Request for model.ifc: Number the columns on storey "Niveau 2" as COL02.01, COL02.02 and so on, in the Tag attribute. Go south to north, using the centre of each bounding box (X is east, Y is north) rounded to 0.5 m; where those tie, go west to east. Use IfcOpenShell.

First a look at what the model holds.

```python
import ifcopenshell
import ifcopenshell.util.element
import ifcopenshell.util.placement

model = ifcopenshell.open("model.ifc")
print(model.schema)
storey = next(s for s in model.by_type("IfcBuildingStorey") if s.Name == "Niveau 2")
columns = [e for e in ifcopenshell.util.element.get_decomposition(storey) if e.is_a("IfcColumn")]
for e in sorted(columns, key=lambda e: e.id()):
    origin = ifcopenshell.util.placement.get_local_placement(e.ObjectPlacement)[:3, 3]
    print(e.id(), e.Tag, e.Name, origin.round(2) + 0.0, sep=" | ")
```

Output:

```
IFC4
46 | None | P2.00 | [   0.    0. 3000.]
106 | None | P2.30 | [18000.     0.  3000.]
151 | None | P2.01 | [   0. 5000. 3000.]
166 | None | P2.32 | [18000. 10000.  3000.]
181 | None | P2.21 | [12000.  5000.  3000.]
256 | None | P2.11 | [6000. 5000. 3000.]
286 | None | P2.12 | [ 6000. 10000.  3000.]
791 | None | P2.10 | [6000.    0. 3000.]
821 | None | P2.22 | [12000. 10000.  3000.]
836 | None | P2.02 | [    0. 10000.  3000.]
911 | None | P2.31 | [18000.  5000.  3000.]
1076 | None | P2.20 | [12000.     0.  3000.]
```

```python
import ifcopenshell
import ifcopenshell.geom
import ifcopenshell.util.element
import ifcopenshell.util.shape

model = ifcopenshell.open("model.ifc")
settings = ifcopenshell.geom.settings()
settings.set("use-world-coords", True)


def centre(element):
    shape = ifcopenshell.geom.create_shape(settings, element)
    return ifcopenshell.util.shape.get_bbox_centroid(shape.geometry)


storey = next(s for s in model.by_type("IfcBuildingStorey") if s.Name == "Niveau 2")
columns = [e for e in ifcopenshell.util.element.get_decomposition(storey) if e.is_a("IfcColumn")]

# Insertion points can sit at a corner or the storey origin, so sort by the geometry (in metres).
centres = {e: centre(e) for e in columns}
columns.sort(key=lambda e: (round(centres[e][1] / 0.5), centres[e][0]))

for i, e in enumerate(columns, start=1):
    number = f"COL02.{i:02d}"
    e.Tag = number
    print(e.id(), number)

model.write("model_updated.ifc")
```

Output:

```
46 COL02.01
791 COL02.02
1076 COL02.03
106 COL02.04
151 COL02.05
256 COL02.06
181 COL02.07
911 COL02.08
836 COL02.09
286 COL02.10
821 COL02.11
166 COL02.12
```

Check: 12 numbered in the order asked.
